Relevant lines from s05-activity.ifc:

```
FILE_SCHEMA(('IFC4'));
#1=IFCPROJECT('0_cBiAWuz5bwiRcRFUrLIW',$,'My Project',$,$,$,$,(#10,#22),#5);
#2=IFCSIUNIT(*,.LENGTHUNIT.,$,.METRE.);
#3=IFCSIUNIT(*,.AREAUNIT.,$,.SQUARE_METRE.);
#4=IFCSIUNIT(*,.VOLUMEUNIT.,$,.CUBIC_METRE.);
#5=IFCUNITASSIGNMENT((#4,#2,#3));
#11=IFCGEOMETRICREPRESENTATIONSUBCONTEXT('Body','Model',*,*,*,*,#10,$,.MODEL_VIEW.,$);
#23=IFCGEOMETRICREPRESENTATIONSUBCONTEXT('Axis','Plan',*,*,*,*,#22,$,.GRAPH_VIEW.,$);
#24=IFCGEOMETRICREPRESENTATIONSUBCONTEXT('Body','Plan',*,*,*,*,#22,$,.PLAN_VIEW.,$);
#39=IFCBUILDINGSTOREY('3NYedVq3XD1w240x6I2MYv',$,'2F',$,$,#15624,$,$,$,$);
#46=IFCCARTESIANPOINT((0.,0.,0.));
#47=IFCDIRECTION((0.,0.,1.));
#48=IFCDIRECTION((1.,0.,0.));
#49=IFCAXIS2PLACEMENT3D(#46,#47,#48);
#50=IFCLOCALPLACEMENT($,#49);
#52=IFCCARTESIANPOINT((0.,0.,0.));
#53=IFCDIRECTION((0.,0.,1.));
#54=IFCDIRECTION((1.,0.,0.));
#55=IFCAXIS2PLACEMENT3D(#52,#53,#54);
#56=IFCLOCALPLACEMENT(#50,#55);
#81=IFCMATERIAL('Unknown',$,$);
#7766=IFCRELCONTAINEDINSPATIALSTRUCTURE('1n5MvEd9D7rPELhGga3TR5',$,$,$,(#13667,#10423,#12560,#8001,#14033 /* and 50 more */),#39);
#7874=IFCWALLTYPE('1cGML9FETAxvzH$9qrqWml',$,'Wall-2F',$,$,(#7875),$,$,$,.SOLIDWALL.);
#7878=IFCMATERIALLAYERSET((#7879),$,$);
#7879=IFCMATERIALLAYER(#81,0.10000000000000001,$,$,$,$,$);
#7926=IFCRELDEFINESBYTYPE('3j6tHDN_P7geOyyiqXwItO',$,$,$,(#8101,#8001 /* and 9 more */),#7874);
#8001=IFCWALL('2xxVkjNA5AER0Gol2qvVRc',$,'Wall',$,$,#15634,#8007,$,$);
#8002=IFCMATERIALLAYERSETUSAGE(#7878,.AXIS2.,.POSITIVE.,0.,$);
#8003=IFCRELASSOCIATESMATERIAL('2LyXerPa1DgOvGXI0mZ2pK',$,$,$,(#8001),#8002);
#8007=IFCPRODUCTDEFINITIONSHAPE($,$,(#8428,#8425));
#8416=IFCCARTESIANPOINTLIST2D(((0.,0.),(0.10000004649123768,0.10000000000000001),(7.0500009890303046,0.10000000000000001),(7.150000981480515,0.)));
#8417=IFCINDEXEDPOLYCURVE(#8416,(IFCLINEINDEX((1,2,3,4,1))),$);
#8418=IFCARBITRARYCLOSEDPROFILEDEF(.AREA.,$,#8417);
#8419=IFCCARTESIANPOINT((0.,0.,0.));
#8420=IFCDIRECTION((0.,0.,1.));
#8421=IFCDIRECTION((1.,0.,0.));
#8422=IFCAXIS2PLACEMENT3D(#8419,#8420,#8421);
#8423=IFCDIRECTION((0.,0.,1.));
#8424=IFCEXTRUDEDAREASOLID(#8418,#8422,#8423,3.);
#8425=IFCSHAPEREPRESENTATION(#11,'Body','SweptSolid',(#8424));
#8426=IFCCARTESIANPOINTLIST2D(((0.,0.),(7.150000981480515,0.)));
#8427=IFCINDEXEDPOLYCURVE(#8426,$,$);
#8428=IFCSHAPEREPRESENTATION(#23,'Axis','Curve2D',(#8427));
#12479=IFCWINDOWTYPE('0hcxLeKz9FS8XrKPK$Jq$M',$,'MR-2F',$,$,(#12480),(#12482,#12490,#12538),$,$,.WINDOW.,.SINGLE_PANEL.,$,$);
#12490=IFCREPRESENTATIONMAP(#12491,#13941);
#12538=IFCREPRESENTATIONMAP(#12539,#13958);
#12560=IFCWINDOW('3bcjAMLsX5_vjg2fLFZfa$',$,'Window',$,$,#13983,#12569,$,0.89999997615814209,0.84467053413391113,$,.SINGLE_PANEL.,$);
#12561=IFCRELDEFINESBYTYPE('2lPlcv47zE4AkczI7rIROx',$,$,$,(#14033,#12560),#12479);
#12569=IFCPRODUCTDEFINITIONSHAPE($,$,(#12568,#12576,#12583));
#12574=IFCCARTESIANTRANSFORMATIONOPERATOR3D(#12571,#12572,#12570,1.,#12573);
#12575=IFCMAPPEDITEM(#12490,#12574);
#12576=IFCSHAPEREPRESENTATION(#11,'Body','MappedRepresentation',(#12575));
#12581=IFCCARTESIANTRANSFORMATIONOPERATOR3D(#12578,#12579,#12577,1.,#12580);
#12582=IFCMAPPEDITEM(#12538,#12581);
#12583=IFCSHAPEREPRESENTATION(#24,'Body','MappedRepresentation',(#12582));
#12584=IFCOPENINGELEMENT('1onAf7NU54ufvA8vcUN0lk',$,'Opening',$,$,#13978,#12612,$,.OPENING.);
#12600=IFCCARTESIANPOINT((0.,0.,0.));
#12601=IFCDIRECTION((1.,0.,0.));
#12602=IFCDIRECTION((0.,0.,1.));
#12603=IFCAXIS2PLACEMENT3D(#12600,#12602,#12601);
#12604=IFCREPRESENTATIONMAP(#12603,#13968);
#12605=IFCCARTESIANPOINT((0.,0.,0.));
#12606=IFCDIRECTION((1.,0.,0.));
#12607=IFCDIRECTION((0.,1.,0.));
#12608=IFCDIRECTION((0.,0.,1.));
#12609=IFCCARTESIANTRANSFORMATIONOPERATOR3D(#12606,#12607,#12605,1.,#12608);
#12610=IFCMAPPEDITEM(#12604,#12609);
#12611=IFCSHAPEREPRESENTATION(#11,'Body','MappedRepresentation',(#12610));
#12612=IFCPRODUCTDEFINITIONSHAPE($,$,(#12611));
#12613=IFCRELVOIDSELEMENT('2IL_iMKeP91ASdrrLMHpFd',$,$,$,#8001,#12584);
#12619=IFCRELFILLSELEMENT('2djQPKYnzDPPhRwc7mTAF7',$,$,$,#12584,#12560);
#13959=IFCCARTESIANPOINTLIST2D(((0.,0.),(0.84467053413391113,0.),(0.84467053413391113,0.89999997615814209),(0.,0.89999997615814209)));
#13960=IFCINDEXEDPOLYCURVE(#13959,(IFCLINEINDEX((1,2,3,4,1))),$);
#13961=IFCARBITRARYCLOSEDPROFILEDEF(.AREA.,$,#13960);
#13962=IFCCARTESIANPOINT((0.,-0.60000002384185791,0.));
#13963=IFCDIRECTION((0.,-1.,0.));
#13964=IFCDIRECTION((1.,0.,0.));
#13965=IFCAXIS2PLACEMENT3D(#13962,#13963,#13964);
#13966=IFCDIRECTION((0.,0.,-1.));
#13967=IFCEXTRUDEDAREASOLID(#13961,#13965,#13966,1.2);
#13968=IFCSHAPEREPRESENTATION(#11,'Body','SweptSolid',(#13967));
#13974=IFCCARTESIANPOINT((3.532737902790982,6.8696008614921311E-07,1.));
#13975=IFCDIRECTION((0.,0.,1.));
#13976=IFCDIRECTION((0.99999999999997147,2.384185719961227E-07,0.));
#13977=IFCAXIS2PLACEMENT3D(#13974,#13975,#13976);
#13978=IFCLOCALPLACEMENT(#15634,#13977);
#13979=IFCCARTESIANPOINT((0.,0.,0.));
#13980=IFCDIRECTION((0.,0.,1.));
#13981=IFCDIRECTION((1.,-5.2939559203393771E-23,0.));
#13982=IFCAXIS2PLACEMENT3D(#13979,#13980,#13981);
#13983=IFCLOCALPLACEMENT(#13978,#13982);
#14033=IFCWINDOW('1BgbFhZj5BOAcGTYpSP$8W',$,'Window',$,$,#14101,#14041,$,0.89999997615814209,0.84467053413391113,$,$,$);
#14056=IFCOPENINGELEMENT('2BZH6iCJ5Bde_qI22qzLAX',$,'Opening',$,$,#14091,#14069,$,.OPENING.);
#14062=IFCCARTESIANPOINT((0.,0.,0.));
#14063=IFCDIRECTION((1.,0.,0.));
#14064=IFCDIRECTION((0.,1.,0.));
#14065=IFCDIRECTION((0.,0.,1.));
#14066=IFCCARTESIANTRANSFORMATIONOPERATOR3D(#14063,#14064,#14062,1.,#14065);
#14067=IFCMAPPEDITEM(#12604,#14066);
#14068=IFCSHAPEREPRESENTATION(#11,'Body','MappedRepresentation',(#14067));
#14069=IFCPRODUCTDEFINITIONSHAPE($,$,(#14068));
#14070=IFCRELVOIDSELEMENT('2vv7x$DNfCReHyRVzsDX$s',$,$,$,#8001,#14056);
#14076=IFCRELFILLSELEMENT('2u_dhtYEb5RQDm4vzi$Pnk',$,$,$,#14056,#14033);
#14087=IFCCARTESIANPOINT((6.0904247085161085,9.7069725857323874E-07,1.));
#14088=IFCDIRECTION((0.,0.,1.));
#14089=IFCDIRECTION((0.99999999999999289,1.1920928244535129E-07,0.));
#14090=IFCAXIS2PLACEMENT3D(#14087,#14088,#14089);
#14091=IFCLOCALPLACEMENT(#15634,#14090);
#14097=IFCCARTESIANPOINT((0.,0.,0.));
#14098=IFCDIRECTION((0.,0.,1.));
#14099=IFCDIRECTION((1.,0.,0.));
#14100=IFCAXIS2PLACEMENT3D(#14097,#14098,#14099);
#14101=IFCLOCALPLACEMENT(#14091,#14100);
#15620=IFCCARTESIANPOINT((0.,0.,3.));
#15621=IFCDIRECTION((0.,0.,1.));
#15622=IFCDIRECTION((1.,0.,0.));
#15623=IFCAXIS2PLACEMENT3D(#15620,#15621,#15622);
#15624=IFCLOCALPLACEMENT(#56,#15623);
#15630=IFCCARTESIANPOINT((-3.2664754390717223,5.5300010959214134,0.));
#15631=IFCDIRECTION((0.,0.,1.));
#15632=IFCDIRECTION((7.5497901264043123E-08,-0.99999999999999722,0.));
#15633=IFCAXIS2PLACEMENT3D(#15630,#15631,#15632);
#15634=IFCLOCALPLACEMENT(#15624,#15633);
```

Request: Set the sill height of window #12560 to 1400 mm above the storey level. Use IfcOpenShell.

```python
import numpy as np
import ifcopenshell
import ifcopenshell.api.geometry
import ifcopenshell.geom
import ifcopenshell.util.element
import ifcopenshell.util.placement
import ifcopenshell.util.shape
import ifcopenshell.util.unit

model = ifcopenshell.open("s05-activity.ifc")
unit_scale = ifcopenshell.util.unit.calculate_unit_scale(model)

window = model.by_id(12560)
opening = window.FillsVoids[0].RelatingOpeningElement
storey = ifcopenshell.util.element.get_container(window, ifc_class="IfcBuildingStorey")
level = ifcopenshell.util.placement.get_local_placement(storey.ObjectPlacement)[2, 3]

# The opening's origin need not be at the sill, so measure its lowest point.
shape = ifcopenshell.geom.create_shape(ifcopenshell.geom.settings(), opening)
bottom = ifcopenshell.util.shape.get_shape_bottom_elevation(shape, shape.geometry) / unit_scale
dz = level + 1.4 - bottom

shift = np.array([0.0, 0.0, dz])
# The window is placed relative to its opening, so it follows when the opening moves.
matrix = ifcopenshell.util.placement.get_local_placement(opening.ObjectPlacement)
matrix[:3, 3] += shift
ifcopenshell.api.geometry.edit_object_placement(
    model, product=opening, matrix=matrix, is_si=False, should_transform_children=True
)

print(f"moved by {dz * unit_scale:+.3f} m")

model.write("s05-activity_v2.ifc")
```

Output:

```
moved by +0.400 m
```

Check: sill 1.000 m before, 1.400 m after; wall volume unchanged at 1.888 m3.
